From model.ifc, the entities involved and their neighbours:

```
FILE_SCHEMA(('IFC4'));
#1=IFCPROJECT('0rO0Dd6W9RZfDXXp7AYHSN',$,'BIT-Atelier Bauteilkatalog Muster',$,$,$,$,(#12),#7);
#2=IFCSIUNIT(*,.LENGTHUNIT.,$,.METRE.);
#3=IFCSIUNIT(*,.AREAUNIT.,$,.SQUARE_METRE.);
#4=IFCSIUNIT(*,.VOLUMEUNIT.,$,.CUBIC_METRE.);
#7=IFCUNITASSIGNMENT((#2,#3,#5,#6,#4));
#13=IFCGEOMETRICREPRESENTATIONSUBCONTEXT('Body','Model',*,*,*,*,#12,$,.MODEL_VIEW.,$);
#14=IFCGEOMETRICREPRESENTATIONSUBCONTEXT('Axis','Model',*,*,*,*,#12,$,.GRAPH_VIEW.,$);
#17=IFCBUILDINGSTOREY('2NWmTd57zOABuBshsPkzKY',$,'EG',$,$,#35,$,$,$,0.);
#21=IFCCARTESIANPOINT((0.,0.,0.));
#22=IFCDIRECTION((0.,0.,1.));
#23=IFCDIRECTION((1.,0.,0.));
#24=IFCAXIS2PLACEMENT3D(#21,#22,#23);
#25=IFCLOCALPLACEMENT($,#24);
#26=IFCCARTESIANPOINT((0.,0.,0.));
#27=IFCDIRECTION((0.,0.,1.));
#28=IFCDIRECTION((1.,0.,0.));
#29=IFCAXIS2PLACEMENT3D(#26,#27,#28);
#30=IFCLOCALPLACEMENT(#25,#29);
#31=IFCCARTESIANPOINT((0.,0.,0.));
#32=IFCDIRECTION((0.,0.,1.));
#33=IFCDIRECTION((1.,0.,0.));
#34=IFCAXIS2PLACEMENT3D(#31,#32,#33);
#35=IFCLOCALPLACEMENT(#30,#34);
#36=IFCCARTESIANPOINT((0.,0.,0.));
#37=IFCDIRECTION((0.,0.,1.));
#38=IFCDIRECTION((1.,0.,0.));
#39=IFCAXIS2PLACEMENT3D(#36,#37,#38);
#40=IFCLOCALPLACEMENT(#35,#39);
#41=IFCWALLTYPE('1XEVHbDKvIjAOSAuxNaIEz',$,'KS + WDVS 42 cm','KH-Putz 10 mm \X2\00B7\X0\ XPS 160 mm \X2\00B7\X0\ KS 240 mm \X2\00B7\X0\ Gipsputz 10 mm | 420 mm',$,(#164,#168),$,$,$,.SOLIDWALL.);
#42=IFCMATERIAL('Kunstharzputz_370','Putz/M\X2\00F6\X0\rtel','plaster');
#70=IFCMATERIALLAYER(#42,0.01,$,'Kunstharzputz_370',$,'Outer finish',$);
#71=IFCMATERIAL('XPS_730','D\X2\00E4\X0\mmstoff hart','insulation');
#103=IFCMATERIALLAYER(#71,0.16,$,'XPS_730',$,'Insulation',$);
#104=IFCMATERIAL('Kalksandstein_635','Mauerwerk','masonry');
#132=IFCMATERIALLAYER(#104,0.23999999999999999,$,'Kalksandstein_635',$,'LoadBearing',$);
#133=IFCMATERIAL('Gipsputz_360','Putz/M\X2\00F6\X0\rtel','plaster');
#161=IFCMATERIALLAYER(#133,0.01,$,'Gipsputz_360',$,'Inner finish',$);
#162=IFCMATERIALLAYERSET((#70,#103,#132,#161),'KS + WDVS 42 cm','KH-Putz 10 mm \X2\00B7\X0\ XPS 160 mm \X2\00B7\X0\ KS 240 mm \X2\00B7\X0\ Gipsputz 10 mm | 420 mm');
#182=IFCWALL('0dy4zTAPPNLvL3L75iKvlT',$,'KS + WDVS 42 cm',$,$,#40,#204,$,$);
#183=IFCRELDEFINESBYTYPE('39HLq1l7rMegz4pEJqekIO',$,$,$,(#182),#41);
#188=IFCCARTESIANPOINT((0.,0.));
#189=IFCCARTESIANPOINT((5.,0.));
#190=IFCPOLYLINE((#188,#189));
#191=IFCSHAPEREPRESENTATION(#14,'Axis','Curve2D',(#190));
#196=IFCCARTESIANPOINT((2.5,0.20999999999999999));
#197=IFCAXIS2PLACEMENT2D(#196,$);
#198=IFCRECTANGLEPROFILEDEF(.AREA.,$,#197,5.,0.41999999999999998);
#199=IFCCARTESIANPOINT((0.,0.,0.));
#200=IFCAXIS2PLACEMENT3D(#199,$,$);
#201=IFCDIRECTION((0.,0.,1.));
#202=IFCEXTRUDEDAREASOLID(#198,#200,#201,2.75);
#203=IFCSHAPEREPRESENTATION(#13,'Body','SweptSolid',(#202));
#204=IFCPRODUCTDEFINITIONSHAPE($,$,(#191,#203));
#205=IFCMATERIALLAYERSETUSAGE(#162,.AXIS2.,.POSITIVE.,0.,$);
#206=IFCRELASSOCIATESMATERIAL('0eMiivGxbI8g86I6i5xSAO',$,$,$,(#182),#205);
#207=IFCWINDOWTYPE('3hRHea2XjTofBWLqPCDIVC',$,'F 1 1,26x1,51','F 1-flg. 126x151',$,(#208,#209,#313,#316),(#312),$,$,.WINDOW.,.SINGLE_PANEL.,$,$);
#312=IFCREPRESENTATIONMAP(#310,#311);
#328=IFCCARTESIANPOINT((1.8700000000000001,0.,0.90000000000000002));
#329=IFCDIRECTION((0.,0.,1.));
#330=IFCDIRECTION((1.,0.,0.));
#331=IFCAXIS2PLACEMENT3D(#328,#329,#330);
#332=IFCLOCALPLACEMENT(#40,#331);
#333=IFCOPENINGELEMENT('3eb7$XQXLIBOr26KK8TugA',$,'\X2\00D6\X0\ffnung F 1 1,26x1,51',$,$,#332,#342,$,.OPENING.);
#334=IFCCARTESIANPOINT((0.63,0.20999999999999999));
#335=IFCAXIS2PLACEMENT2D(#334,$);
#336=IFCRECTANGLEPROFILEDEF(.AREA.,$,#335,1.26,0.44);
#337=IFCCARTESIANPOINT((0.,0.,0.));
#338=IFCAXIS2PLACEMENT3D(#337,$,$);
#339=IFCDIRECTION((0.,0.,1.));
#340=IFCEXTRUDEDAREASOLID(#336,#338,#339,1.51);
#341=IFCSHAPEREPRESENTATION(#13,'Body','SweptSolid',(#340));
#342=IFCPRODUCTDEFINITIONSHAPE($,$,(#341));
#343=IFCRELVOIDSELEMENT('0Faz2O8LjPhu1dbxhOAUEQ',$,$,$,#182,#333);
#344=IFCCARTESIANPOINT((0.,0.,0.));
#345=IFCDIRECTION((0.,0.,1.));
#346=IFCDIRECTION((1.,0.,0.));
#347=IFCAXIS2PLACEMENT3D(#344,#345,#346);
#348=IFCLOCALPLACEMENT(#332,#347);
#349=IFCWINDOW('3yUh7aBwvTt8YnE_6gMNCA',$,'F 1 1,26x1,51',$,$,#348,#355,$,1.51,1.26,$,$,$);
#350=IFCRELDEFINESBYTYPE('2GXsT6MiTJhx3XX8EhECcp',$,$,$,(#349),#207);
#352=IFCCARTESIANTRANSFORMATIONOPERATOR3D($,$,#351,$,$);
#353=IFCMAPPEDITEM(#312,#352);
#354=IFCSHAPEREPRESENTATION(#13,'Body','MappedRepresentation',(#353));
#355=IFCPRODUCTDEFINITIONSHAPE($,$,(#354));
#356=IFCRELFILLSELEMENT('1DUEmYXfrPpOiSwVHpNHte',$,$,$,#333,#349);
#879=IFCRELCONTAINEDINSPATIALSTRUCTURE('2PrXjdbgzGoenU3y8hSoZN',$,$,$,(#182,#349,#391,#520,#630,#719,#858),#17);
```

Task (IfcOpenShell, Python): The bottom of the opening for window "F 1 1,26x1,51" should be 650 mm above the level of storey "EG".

```python
import numpy as np
import ifcopenshell
import ifcopenshell.api.geometry
import ifcopenshell.geom
import ifcopenshell.util.element
import ifcopenshell.util.placement
import ifcopenshell.util.shape
import ifcopenshell.util.unit

model = ifcopenshell.open("model.ifc")
unit_scale = ifcopenshell.util.unit.calculate_unit_scale(model)

window = model.by_guid("3yUh7aBwvTt8YnE_6gMNCA")
opening = window.FillsVoids[0].RelatingOpeningElement
storey = ifcopenshell.util.element.get_container(window, ifc_class="IfcBuildingStorey")
level = ifcopenshell.util.placement.get_local_placement(storey.ObjectPlacement)[2, 3]

# The opening's origin need not be at the sill, so measure its lowest point.
shape = ifcopenshell.geom.create_shape(ifcopenshell.geom.settings(), opening)
bottom = ifcopenshell.util.shape.get_shape_bottom_elevation(shape, shape.geometry) / unit_scale
dz = level + 0.65 / unit_scale - bottom

shift = np.array([0.0, 0.0, dz])
# The window is placed relative to its opening, so it follows when the opening moves.
matrix = ifcopenshell.util.placement.get_local_placement(opening.ObjectPlacement)
matrix[:3, 3] += shift
ifcopenshell.api.geometry.edit_object_placement(
    model, product=opening, matrix=matrix, is_si=False, should_transform_children=True
)

print(f"moved by {dz * unit_scale:+.3f} m")

model.write("model_updated.ifc")
```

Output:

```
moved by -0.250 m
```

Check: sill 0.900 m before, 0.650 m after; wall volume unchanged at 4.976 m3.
